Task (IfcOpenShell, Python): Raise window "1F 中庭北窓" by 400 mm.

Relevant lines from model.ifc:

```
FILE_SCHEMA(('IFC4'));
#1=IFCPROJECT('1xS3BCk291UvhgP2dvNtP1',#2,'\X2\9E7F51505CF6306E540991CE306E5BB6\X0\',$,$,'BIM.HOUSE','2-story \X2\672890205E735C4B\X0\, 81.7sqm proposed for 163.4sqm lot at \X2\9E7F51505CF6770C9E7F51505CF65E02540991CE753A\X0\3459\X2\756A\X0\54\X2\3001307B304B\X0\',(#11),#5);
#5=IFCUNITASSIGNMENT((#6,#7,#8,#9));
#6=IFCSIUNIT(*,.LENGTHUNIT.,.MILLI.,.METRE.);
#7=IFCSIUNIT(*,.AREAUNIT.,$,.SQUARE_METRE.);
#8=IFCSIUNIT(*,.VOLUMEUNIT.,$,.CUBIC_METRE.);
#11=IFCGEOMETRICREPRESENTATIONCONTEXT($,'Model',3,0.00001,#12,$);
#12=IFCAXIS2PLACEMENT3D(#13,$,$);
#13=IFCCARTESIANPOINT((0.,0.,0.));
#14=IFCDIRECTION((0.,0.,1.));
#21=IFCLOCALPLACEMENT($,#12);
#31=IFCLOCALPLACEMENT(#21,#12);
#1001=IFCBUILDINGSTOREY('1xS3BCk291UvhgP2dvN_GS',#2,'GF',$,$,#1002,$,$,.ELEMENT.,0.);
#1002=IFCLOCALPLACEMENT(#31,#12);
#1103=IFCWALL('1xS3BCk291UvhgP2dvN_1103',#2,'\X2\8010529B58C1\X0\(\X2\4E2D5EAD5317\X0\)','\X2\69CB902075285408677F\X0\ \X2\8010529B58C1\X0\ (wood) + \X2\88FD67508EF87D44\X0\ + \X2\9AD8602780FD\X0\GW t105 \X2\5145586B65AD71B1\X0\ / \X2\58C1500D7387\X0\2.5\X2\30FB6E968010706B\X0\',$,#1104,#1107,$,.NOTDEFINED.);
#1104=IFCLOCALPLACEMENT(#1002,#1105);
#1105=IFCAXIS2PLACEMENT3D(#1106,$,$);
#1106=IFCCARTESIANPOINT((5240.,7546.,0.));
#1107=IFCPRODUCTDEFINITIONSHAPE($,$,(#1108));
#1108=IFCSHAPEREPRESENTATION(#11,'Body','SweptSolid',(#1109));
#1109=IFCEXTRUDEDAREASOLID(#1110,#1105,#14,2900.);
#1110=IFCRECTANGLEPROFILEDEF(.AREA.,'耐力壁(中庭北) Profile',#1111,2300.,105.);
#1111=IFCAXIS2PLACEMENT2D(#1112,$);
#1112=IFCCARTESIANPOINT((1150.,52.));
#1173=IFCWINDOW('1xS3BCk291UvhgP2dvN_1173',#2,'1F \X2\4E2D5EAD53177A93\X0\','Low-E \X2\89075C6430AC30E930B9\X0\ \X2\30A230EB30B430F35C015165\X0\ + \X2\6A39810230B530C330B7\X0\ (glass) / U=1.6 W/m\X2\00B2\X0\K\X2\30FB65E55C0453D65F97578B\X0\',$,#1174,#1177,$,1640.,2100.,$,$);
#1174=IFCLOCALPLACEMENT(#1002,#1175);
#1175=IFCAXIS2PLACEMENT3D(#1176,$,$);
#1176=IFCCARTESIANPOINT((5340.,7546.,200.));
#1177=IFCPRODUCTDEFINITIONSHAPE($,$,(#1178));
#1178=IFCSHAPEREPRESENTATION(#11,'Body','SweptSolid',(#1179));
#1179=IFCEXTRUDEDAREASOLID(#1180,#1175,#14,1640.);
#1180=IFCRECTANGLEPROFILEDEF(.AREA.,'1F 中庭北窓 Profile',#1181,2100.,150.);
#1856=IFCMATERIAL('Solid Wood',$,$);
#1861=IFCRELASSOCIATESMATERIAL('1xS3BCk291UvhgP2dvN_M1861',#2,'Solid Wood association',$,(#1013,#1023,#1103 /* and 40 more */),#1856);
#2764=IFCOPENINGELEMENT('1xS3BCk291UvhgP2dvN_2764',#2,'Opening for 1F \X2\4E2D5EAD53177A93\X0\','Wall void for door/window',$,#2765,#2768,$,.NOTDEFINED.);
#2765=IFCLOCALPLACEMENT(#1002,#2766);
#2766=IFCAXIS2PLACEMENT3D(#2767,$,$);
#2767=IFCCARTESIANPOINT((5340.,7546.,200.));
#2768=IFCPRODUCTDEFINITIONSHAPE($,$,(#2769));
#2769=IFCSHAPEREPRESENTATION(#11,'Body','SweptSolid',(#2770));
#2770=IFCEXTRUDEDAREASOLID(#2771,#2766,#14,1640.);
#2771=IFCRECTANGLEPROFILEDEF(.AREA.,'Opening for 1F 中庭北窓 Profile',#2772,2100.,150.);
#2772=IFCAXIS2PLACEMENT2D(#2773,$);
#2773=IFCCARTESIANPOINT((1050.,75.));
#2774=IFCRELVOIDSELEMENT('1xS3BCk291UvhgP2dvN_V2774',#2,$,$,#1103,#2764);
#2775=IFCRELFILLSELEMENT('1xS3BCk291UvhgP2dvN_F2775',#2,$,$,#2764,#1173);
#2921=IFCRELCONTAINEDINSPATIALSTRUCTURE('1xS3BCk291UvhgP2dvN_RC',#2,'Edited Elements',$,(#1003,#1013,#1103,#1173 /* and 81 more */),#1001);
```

```python
import numpy as np
import ifcopenshell
import ifcopenshell.api.geometry
import ifcopenshell.util.placement
import ifcopenshell.util.unit

model = ifcopenshell.open("model.ifc")
unit_scale = ifcopenshell.util.unit.calculate_unit_scale(model)

window = model.by_id(1173)
opening = window.FillsVoids[0].RelatingOpeningElement
dz = 0.4 / unit_scale

shift = np.array([0.0, 0.0, dz])
# The window is not placed relative to its opening, so move both.
for product in (opening, window):
    matrix = ifcopenshell.util.placement.get_local_placement(product.ObjectPlacement)
    matrix[:3, 3] += shift
    ifcopenshell.api.geometry.edit_object_placement(model, product=product, matrix=matrix, is_si=False)

print(f"moved by {dz * unit_scale:+.3f} m")

model.write("model-out.ifc")
```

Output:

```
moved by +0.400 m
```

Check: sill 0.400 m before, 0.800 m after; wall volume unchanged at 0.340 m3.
